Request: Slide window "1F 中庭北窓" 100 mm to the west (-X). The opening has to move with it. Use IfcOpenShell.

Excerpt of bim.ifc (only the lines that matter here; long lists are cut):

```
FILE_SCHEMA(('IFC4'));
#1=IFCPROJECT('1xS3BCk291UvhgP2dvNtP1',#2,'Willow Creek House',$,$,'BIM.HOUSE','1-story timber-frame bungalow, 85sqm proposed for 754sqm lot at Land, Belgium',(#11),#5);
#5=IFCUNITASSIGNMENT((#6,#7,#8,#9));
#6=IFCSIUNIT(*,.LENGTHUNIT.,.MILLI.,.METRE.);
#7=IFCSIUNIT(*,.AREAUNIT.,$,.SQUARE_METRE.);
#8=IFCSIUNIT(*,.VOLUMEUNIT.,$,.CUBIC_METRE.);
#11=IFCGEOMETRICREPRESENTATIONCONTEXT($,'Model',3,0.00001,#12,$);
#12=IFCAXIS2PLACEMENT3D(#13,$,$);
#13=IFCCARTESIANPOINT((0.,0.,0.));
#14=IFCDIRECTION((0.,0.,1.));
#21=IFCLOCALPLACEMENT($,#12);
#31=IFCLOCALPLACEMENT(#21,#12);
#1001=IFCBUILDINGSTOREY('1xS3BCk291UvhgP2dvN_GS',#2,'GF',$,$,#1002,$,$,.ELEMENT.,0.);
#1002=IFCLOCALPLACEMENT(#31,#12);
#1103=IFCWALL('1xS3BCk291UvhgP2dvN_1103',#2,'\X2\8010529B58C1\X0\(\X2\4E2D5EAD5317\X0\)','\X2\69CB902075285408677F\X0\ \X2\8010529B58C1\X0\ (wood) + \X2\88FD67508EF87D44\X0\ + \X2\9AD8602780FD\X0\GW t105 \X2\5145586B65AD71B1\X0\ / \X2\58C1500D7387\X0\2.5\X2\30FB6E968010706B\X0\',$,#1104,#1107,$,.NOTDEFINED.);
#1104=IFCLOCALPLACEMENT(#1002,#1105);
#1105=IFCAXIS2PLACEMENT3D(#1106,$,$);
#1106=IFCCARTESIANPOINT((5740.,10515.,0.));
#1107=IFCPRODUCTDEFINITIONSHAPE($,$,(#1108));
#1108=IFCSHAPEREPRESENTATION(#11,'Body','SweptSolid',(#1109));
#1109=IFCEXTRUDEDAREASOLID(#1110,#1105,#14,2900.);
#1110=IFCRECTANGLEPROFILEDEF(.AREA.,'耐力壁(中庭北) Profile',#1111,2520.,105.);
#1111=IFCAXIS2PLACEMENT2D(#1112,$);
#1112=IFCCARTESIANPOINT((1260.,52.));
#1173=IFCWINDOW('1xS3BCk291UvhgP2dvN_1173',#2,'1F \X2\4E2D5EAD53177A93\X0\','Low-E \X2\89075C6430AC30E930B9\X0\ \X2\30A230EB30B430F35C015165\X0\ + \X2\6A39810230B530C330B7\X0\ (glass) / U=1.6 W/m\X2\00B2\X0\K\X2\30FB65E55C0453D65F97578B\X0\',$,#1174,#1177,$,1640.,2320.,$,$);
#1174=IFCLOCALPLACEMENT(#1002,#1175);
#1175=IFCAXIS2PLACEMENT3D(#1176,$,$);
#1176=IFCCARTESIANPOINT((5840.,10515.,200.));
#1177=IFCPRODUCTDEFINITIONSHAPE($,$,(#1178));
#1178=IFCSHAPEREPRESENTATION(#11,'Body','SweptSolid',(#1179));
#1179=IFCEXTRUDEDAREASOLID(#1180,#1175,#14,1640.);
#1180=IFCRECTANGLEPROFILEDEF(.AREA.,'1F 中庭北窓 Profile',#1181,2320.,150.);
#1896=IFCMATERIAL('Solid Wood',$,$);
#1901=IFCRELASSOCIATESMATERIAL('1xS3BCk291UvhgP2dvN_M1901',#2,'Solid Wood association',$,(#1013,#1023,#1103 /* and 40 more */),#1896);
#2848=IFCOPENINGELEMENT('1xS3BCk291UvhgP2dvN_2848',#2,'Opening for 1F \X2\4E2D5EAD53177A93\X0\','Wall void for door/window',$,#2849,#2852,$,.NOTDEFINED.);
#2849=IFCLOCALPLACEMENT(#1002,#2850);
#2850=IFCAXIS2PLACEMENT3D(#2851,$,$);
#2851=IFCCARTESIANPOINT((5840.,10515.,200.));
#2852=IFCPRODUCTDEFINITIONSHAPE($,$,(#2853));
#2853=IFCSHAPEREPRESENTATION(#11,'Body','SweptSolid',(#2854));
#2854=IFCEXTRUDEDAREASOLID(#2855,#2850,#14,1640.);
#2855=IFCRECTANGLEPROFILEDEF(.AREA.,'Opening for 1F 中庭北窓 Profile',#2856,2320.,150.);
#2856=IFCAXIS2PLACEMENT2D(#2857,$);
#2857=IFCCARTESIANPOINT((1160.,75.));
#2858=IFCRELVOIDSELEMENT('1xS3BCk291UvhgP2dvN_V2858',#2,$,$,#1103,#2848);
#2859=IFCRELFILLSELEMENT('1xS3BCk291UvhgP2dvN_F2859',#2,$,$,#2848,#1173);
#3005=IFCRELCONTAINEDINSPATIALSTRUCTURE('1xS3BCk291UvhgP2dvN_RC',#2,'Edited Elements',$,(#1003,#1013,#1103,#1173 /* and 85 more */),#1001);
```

```python
import ifcopenshell
import ifcopenshell.api.geometry
import ifcopenshell.util.placement
import ifcopenshell.util.unit

model = ifcopenshell.open("bim.ifc")
unit_scale = ifcopenshell.util.unit.calculate_unit_scale(model)

window = model.by_id(1173)
opening = window.FillsVoids[0].RelatingOpeningElement
wall = opening.VoidsElements[0].RelatingBuildingElement

wall_matrix = ifcopenshell.util.placement.get_local_placement(wall.ObjectPlacement)
shift = wall_matrix[:3, 0] * -0.1 / unit_scale
before = ifcopenshell.util.placement.get_local_placement(window.ObjectPlacement)[:3, 3].copy()

# The window is not placed relative to its opening, so move both.
for product in (opening, window):
    matrix = ifcopenshell.util.placement.get_local_placement(product.ObjectPlacement)
    matrix[:3, 3] += shift
    ifcopenshell.api.geometry.edit_object_placement(model, product=product, matrix=matrix, is_si=False)

after = ifcopenshell.util.placement.get_local_placement(window.ObjectPlacement)[:3, 3]
print("window moved by", (after - before).round(3) + 0.0)

model.write("bim_updated.ifc")
```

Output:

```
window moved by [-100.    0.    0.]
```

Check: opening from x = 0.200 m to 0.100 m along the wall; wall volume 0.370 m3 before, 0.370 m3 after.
